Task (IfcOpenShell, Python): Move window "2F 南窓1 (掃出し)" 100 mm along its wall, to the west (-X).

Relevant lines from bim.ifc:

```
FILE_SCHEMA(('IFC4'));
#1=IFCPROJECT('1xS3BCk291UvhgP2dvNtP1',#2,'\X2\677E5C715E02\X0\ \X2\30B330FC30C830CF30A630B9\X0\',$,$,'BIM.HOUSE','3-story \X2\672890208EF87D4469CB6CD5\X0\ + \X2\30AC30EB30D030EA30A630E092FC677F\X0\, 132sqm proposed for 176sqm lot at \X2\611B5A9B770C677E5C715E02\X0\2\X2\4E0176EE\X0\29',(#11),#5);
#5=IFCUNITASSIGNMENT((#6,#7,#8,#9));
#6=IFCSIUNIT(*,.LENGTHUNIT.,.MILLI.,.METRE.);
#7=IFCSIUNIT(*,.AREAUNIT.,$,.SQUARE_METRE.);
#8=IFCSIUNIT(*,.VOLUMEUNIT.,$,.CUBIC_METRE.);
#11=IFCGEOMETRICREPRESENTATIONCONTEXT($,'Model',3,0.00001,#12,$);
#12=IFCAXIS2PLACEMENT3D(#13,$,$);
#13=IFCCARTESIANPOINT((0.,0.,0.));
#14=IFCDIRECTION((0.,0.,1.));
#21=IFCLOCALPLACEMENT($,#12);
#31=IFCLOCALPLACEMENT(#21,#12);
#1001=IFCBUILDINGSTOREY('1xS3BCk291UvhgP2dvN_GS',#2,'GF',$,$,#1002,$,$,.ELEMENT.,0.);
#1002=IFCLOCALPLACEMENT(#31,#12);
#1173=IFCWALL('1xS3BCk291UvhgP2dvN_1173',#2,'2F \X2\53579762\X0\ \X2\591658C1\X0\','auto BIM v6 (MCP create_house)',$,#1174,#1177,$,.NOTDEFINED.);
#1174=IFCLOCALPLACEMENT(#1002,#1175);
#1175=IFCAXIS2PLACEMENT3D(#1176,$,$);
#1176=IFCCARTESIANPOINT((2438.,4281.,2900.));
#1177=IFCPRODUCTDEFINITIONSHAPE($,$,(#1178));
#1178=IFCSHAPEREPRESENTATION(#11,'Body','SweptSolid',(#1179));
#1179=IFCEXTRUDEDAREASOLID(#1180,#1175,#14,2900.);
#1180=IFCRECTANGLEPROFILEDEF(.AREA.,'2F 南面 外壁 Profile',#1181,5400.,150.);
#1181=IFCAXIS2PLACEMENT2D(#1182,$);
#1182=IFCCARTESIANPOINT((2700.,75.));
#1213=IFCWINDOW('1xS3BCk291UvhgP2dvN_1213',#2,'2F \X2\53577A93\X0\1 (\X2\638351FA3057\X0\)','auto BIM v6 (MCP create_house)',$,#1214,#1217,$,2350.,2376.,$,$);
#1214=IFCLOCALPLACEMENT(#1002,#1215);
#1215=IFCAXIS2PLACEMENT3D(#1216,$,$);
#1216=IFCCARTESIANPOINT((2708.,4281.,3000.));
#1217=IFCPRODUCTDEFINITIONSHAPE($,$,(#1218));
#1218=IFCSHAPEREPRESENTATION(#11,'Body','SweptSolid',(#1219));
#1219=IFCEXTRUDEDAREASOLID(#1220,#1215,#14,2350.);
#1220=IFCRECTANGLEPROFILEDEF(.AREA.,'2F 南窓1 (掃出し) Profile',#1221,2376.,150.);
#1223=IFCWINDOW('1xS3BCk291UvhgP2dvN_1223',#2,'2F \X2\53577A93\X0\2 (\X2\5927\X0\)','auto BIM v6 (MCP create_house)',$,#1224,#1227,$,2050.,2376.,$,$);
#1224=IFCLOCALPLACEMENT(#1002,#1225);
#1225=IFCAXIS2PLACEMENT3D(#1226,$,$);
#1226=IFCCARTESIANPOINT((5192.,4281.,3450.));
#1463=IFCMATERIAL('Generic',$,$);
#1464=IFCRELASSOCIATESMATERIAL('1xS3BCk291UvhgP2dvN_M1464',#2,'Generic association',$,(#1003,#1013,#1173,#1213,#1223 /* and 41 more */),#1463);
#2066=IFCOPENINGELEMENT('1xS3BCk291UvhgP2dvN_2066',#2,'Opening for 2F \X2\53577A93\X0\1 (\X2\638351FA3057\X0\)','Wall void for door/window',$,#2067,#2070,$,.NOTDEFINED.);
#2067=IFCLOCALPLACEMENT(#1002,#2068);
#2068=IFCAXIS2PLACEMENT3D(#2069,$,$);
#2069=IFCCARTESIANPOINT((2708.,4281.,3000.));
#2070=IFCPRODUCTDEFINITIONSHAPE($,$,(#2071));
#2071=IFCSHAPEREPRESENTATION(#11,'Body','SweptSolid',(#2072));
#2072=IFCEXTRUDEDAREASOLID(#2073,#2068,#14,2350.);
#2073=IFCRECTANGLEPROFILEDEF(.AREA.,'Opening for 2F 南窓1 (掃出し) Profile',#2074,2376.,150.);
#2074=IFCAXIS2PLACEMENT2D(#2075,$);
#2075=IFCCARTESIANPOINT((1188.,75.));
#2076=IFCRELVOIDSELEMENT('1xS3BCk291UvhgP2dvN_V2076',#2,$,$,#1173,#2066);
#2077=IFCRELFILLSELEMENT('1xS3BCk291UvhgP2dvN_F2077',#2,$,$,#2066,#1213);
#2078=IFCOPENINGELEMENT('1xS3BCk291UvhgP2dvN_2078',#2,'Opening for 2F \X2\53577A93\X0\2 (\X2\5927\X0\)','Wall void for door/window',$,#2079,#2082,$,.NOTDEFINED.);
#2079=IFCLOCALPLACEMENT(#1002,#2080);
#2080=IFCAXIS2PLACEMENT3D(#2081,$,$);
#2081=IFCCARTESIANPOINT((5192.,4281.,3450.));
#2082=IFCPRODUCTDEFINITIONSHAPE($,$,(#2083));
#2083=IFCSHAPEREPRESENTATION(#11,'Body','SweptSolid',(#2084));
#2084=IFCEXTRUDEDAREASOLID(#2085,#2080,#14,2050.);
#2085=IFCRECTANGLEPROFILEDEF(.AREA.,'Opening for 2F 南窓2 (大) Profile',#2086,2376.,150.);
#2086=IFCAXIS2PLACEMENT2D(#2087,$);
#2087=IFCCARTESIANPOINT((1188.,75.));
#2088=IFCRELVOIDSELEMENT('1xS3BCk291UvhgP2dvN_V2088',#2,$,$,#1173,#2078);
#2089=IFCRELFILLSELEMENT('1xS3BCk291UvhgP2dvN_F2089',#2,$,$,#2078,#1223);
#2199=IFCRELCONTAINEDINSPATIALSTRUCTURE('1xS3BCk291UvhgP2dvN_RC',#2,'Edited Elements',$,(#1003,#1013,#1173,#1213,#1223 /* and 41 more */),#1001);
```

```python
import ifcopenshell
import ifcopenshell.api.geometry
import ifcopenshell.util.placement

model = ifcopenshell.open("bim.ifc")

window = model.by_id(1213)
opening = window.FillsVoids[0].RelatingOpeningElement
wall = opening.VoidsElements[0].RelatingBuildingElement

wall_matrix = ifcopenshell.util.placement.get_local_placement(wall.ObjectPlacement)
shift = wall_matrix[:3, 0] * -100.0
before = ifcopenshell.util.placement.get_local_placement(window.ObjectPlacement)[:3, 3].copy()

# The window is not placed relative to its opening, so move both.
for product in (opening, window):
    matrix = ifcopenshell.util.placement.get_local_placement(product.ObjectPlacement)
    matrix[:3, 3] += shift
    ifcopenshell.api.geometry.edit_object_placement(model, product=product, matrix=matrix, is_si=False)

after = ifcopenshell.util.placement.get_local_placement(window.ObjectPlacement)[:3, 3]
print("window moved by", (after - before).round(3) + 0.0)

model.write("bim_rev.ifc")
```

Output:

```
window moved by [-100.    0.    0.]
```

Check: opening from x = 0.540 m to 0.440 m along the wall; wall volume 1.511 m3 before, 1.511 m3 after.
